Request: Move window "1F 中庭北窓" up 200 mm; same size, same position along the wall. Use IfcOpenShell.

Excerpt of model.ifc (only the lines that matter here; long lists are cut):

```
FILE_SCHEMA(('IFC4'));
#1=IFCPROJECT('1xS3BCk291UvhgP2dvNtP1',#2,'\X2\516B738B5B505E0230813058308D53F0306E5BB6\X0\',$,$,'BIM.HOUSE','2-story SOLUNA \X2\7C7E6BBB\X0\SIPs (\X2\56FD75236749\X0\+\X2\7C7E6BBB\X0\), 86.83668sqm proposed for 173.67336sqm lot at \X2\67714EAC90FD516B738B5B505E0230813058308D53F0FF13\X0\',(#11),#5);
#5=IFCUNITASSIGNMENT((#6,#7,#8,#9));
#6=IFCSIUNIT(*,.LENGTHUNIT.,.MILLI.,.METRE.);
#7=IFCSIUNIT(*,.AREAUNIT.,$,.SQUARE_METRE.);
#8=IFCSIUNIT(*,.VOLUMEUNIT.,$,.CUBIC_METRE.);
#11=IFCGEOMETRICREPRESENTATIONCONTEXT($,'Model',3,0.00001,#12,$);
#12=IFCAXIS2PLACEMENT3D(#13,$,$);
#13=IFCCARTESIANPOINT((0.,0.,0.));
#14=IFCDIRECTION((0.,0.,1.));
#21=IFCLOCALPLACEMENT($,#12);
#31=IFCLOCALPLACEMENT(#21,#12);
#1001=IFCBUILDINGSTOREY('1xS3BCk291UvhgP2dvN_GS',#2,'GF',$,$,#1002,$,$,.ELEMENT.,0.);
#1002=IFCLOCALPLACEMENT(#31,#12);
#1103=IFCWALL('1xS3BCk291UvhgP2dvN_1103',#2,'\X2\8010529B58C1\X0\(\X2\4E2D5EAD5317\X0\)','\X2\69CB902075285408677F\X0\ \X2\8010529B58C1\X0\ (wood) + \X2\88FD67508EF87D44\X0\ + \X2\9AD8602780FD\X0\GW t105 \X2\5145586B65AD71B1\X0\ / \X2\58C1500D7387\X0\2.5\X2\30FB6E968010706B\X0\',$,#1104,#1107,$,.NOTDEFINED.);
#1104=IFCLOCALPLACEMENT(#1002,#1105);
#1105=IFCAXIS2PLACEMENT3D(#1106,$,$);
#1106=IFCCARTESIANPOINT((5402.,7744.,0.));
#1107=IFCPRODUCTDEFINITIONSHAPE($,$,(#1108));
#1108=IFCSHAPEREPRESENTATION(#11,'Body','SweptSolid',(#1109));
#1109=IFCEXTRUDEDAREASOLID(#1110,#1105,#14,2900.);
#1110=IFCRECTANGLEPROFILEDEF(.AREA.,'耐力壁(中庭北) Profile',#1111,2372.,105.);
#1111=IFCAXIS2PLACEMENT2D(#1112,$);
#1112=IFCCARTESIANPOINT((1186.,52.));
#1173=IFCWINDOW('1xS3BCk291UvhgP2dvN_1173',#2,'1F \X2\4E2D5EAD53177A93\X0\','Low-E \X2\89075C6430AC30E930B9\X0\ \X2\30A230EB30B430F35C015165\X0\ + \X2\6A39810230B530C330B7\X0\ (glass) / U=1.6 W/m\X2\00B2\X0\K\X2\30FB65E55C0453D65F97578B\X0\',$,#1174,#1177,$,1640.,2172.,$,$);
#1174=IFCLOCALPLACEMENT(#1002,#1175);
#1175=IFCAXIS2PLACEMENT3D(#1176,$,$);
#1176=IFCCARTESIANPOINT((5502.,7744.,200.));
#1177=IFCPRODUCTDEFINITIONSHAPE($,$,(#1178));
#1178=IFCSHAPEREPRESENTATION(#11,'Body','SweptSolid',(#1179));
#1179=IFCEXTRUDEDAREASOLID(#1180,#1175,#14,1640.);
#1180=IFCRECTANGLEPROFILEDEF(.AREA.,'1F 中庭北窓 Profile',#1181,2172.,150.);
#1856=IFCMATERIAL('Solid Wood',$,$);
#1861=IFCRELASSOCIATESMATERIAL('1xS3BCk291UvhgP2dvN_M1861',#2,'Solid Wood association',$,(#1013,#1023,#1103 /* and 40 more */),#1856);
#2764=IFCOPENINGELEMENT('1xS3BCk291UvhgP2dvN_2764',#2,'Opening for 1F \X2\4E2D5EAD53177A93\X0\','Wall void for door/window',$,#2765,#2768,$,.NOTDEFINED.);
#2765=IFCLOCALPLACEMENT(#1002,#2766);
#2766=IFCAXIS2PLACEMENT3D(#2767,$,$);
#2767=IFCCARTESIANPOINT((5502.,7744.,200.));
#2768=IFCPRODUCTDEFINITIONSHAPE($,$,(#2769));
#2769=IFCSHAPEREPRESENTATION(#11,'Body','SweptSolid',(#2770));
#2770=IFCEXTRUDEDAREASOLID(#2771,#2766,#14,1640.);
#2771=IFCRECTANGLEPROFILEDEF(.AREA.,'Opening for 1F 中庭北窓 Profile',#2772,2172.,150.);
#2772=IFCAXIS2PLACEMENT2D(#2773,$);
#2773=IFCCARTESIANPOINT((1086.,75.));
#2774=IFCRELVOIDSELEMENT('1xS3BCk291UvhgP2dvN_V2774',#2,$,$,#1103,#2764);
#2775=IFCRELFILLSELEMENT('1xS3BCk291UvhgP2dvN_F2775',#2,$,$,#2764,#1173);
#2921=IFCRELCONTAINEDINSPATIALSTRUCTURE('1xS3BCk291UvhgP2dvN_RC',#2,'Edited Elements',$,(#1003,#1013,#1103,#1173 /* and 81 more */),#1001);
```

```python
import numpy as np
import ifcopenshell
import ifcopenshell.api.geometry
import ifcopenshell.util.placement
import ifcopenshell.util.unit

model = ifcopenshell.open("model.ifc")
unit_scale = ifcopenshell.util.unit.calculate_unit_scale(model)

window = model.by_guid("1xS3BCk291UvhgP2dvN_1173")
opening = window.FillsVoids[0].RelatingOpeningElement
dz = 200.0

shift = np.array([0.0, 0.0, dz])
# The window is not placed relative to its opening, so move both.
for product in (opening, window):
    matrix = ifcopenshell.util.placement.get_local_placement(product.ObjectPlacement)
    matrix[:3, 3] += shift
    ifcopenshell.api.geometry.edit_object_placement(model, product=product, matrix=matrix, is_si=False)

print(f"moved by {dz * unit_scale:+.3f} m")

model.write("model_updated.ifc")
```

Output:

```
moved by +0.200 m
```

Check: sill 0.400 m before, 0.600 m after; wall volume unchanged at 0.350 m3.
